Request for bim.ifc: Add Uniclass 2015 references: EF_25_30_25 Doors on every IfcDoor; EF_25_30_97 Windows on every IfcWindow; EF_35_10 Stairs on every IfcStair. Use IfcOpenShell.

First a look at what the model holds.

```python
import ifcopenshell

model = ifcopenshell.open("bim.ifc")
print(model.schema)
print("classifications:", [c.Name for c in model.by_type("IfcClassification")])
for ifc_class in ("IfcDoor", "IfcRoof", "IfcStair", "IfcWall", "IfcWindow"):
    print(ifc_class, len(model.by_type(ifc_class)))
```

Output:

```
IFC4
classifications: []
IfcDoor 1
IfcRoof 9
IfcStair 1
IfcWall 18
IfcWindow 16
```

```python
import ifcopenshell
import ifcopenshell.api.classification

model = ifcopenshell.open("bim.ifc")

system = ifcopenshell.api.classification.add_classification(model, classification="Uniclass 2015")

codes = {
    "IfcDoor": ("EF_25_30_25", "Doors"),
    "IfcWindow": ("EF_25_30_97", "Windows"),
    "IfcStair": ("EF_35_10", "Stairs"),
}
for ifc_class, (code, name) in codes.items():
    products = model.by_type(ifc_class)
    ifcopenshell.api.classification.add_reference(
        model, products=products, classification=system, identification=code, name=name
    )
    print(code, len(products))

model.write("bim_v2.ifc")
```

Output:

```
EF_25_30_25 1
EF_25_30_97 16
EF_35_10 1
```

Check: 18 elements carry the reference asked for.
